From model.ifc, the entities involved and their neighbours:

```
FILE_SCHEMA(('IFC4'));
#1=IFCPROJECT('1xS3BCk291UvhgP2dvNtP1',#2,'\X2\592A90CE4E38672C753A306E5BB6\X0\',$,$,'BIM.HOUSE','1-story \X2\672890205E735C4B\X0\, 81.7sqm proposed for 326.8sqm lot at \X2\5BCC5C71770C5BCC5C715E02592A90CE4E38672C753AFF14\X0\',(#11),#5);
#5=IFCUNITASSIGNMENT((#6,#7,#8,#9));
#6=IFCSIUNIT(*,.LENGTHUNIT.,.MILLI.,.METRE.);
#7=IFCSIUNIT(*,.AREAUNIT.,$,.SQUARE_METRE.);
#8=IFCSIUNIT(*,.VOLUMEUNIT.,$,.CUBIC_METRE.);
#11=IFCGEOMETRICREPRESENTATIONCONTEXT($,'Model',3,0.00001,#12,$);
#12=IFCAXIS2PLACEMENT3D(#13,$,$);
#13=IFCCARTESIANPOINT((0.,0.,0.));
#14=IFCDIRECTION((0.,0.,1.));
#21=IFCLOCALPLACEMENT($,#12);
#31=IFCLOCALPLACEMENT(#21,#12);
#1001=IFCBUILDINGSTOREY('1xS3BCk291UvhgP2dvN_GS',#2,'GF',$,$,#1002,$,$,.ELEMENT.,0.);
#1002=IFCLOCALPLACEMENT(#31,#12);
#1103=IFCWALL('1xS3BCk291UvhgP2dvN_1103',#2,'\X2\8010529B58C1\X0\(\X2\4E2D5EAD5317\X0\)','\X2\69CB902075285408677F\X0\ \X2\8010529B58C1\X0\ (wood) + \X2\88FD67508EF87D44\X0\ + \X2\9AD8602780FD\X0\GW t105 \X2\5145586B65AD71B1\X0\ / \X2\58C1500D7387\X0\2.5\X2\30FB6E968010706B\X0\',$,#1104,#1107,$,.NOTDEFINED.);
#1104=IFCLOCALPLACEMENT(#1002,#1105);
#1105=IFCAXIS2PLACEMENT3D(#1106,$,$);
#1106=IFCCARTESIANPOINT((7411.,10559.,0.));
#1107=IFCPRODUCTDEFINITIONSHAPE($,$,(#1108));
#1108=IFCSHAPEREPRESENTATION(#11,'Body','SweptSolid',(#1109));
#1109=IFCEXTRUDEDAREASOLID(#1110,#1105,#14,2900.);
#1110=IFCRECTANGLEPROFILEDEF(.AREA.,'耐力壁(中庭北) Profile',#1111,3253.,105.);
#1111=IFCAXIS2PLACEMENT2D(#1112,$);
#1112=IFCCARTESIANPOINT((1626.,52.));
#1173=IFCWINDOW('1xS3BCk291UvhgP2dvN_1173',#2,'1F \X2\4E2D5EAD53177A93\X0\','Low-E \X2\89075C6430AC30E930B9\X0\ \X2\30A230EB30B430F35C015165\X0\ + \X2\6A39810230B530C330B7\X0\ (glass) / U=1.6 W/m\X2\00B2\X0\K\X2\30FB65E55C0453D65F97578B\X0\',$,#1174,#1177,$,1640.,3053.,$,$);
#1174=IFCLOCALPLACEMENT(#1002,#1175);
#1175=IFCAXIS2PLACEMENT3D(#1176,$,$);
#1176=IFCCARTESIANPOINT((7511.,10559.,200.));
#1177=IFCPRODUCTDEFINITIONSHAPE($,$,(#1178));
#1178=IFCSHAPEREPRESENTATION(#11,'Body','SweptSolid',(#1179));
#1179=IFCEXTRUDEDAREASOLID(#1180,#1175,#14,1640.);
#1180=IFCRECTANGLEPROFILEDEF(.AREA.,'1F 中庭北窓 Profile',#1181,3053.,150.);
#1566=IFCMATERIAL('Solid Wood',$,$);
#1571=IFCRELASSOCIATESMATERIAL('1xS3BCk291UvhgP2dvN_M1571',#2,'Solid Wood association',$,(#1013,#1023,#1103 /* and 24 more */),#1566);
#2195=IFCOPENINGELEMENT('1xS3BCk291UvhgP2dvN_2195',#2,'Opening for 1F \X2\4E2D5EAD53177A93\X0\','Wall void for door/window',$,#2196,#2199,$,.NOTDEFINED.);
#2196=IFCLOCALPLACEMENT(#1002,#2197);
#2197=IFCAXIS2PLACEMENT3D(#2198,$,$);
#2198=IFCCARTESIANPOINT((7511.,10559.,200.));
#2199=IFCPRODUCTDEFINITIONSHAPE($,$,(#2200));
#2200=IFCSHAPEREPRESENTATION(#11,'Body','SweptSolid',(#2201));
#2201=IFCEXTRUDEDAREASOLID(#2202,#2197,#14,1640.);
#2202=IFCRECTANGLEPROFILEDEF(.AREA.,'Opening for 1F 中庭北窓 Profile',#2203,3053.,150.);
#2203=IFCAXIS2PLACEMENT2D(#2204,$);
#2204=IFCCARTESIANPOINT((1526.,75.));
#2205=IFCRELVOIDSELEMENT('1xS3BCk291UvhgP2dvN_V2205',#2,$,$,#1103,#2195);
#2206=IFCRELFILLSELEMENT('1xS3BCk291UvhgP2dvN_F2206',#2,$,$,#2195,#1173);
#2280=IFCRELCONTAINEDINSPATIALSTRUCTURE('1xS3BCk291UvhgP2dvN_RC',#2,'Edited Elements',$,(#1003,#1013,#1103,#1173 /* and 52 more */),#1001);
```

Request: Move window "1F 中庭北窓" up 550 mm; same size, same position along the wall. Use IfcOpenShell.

```python
import numpy as np
import ifcopenshell
import ifcopenshell.api.geometry
import ifcopenshell.util.placement
import ifcopenshell.util.unit

model = ifcopenshell.open("model.ifc")
unit_scale = ifcopenshell.util.unit.calculate_unit_scale(model)

window = model.by_guid("1xS3BCk291UvhgP2dvN_1173")
opening = window.FillsVoids[0].RelatingOpeningElement
dz = 0.55 / unit_scale

shift = np.array([0.0, 0.0, dz])
# The window is not placed relative to its opening, so move both.
for product in (opening, window):
    matrix = ifcopenshell.util.placement.get_local_placement(product.ObjectPlacement)
    matrix[:3, 3] += shift
    ifcopenshell.api.geometry.edit_object_placement(model, product=product, matrix=matrix, is_si=False)

print(f"moved by {dz * unit_scale:+.3f} m")

model.write("model_v2.ifc")
```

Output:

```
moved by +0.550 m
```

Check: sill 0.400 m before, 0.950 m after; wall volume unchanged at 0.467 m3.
